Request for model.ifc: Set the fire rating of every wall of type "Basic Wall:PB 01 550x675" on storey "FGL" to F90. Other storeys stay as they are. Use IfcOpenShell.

First a look at what the model holds.

```python
import ifcopenshell
import ifcopenshell.util.element

model = ifcopenshell.open("model.ifc")
print(model.schema)
storey = next(s for s in model.by_type("IfcBuildingStorey") if s.Name == "FGL")
walls = [e for e in ifcopenshell.util.element.get_decomposition(storey) if e.is_a("IfcWall")]
seen = {}
for e in walls:
    element_type = ifcopenshell.util.element.get_type(e)
    key = (element_type.Name if element_type != e and element_type else None, ifcopenshell.util.element.get_pset(e, "Pset_WallCommon", "FireRating"))
    seen[key] = seen.get(key, 0) + 1
for (name, value), count in sorted(seen.items(), key=str):
    print(count, "x", name, "|", value)
```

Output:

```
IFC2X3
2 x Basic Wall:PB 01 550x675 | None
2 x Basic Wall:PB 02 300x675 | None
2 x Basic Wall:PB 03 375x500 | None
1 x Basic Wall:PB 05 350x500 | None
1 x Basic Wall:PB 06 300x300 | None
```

```python
import ifcopenshell
import ifcopenshell.api.pset
import ifcopenshell.util.element

model = ifcopenshell.open("model.ifc")

storey = next(s for s in model.by_type("IfcBuildingStorey") if s.Name == "FGL")
walls = [e for e in ifcopenshell.util.element.get_decomposition(storey) if e.is_a("IfcWall")]

count = 0
for e in walls:
    element_type = ifcopenshell.util.element.get_type(e)
    if element_type in (None, e) or element_type.Name != "Basic Wall:PB 01 550x675":
        continue
    # add_pset returns the element's existing set when there is one.
    pset = ifcopenshell.api.pset.add_pset(model, product=e, name="Pset_WallCommon")
    ifcopenshell.api.pset.edit_pset(model, pset=pset, properties={"FireRating": "F90"})
    count += 1

print(count, "walls updated")

model.write("model_rev.ifc")
```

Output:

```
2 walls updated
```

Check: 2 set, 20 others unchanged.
